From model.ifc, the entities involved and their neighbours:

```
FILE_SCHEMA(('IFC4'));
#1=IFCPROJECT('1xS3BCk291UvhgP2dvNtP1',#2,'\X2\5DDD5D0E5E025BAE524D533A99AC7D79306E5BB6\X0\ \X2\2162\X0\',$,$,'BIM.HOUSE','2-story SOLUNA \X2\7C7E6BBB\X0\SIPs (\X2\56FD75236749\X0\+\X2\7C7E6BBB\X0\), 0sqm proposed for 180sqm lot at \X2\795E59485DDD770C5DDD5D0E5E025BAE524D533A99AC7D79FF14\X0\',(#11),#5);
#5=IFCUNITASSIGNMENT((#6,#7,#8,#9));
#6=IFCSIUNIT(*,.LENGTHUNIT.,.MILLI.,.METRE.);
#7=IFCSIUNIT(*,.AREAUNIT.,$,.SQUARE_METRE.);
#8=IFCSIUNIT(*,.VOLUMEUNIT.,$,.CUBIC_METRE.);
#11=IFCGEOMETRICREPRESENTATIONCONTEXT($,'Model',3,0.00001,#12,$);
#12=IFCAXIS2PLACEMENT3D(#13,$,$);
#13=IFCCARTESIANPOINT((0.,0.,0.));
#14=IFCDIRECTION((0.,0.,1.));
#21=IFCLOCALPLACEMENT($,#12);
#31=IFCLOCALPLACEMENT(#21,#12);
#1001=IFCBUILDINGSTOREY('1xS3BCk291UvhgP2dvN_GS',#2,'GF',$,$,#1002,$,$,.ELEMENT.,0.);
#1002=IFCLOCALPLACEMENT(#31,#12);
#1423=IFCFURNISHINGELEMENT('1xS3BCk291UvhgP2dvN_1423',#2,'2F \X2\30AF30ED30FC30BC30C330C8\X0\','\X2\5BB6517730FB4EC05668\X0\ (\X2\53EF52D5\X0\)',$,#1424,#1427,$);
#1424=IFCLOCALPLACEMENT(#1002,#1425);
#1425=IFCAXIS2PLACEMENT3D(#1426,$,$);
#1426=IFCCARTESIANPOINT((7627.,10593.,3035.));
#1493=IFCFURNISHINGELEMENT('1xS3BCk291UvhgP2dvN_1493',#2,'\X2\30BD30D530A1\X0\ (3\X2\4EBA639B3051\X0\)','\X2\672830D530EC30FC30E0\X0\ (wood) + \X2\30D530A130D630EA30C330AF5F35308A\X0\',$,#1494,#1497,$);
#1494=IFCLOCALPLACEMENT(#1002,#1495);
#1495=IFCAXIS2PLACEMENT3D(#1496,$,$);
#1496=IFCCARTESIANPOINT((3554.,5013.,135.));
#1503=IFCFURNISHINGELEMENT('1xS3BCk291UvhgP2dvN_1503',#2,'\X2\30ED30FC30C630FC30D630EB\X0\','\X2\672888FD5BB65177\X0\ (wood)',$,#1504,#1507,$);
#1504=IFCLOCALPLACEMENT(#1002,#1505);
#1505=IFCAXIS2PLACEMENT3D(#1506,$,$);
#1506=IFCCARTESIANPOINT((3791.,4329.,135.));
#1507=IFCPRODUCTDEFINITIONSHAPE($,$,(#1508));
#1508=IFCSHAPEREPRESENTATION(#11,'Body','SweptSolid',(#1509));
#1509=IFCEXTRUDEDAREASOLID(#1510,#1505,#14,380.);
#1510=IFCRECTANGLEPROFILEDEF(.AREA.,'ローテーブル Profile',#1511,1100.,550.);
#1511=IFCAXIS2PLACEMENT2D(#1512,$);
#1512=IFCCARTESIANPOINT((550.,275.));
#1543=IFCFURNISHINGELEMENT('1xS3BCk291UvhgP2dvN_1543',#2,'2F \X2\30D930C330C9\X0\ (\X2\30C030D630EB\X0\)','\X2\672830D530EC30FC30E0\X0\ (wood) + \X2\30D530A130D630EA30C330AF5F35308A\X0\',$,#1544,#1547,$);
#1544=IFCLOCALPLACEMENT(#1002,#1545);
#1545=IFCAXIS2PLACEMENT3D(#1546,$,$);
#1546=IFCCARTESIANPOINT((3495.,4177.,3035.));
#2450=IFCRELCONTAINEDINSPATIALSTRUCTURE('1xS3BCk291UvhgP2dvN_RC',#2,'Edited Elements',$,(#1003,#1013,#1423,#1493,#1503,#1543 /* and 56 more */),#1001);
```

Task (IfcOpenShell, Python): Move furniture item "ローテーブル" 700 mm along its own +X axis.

```python
import ifcopenshell
import ifcopenshell.api.geometry
import ifcopenshell.util.placement

model = ifcopenshell.open("model.ifc")

item = model.by_guid("1xS3BCk291UvhgP2dvN_1503")
matrix = ifcopenshell.util.placement.get_local_placement(item.ObjectPlacement)
matrix[:3, 3] += matrix[:3, 0] * 700.0
ifcopenshell.api.geometry.edit_object_placement(model, product=item, matrix=matrix, is_si=False)

print(ifcopenshell.util.placement.get_local_placement(item.ObjectPlacement).round(3) + 0.0)

model.write("model_rev.ifc")
```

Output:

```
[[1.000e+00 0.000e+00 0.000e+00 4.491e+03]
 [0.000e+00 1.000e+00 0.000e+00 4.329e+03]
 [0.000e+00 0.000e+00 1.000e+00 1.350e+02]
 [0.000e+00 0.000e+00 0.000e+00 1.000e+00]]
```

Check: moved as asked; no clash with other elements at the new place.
